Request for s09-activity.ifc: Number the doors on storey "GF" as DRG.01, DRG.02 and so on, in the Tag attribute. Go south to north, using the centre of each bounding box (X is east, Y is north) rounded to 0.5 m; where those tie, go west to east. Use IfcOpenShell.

First a look at what the model holds.

```python
import ifcopenshell
import ifcopenshell.util.element
import ifcopenshell.util.placement

model = ifcopenshell.open("s09-activity.ifc")
print(model.schema)
storey = next(s for s in model.by_type("IfcBuildingStorey") if s.Name == "GF")
doors = [e for e in ifcopenshell.util.element.get_decomposition(storey) if e.is_a("IfcDoor")]
for e in sorted(doors, key=lambda e: e.id()):
    origin = ifcopenshell.util.placement.get_local_placement(e.ObjectPlacement)[:3, 3]
    print(e.id(), e.Tag, e.Name, origin.round(2) + 0.0, sep=" | ")
```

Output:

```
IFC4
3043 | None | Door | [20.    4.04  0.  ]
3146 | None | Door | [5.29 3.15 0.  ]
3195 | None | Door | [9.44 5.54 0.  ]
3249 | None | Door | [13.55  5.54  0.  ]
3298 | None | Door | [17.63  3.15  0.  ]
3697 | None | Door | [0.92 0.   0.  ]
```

```python
import ifcopenshell
import ifcopenshell.geom
import ifcopenshell.util.element
import ifcopenshell.util.shape

model = ifcopenshell.open("s09-activity.ifc")
settings = ifcopenshell.geom.settings()
settings.set("use-world-coords", True)


def centre(element):
    shape = ifcopenshell.geom.create_shape(settings, element)
    return ifcopenshell.util.shape.get_bbox_centroid(shape.geometry)


storey = next(s for s in model.by_type("IfcBuildingStorey") if s.Name == "GF")
doors = [e for e in ifcopenshell.util.element.get_decomposition(storey) if e.is_a("IfcDoor")]

# Insertion points can sit at a corner or the storey origin, so sort by the geometry (in metres).
centres = {e: centre(e) for e in doors}
doors.sort(key=lambda e: (round(centres[e][1] / 0.5), centres[e][0]))

for i, e in enumerate(doors, start=1):
    number = f"DRG.{i:02d}"
    e.Tag = number
    print(e.id(), number)

model.write("s09-activity_updated.ifc")
```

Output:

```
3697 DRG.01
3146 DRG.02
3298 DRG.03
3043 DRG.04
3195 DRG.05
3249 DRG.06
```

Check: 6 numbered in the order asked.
